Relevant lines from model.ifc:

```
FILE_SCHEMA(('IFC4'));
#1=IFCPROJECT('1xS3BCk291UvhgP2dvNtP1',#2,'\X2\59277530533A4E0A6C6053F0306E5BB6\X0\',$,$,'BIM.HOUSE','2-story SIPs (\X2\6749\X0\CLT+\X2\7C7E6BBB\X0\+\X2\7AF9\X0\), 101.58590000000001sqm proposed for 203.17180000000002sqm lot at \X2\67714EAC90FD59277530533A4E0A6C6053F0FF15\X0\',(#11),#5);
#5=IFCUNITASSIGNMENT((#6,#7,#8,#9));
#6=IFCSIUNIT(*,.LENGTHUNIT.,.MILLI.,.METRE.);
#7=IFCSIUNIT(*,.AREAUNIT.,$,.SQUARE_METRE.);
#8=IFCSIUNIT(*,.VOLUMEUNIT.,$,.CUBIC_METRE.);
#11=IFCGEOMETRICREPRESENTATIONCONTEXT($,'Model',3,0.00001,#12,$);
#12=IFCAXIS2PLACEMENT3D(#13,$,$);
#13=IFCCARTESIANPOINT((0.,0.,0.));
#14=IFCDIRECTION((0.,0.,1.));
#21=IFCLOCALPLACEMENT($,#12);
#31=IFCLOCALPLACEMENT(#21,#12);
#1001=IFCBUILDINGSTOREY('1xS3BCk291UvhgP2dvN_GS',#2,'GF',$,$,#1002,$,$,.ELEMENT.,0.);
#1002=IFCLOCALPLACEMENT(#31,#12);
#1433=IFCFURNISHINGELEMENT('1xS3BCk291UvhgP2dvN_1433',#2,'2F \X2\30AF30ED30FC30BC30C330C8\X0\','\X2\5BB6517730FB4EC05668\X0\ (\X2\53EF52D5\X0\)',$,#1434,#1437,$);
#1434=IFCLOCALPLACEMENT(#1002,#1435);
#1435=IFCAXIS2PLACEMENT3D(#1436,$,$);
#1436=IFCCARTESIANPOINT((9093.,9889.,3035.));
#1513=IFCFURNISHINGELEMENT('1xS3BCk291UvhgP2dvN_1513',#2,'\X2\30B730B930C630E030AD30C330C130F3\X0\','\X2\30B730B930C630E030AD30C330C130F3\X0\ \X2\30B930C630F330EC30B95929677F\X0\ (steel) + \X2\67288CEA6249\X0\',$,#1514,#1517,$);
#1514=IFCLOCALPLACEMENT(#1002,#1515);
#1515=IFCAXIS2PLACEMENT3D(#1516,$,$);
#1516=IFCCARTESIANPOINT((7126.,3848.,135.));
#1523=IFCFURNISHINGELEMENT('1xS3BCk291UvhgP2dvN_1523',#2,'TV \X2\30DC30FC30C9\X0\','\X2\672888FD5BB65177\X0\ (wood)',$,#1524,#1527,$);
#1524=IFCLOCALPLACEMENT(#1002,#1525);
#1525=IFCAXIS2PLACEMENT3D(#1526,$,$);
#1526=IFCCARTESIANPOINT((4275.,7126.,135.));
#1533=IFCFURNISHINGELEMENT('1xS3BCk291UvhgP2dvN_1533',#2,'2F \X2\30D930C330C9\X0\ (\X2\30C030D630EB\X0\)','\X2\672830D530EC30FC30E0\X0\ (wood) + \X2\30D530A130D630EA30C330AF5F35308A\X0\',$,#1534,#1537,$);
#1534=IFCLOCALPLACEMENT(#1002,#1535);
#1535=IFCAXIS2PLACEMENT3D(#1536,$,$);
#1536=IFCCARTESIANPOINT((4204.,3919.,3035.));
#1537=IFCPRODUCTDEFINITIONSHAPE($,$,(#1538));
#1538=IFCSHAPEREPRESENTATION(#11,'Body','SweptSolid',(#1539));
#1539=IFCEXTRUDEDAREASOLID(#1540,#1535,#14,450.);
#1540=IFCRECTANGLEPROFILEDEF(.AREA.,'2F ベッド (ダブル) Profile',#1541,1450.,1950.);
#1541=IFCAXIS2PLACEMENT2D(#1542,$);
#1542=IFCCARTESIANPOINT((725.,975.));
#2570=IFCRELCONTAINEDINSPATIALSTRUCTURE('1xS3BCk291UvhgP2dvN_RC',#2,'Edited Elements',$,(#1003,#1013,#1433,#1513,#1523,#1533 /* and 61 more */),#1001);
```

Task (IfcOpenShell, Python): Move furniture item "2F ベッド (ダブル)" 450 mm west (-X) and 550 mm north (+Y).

```python
import ifcopenshell
import ifcopenshell.api.geometry
import ifcopenshell.util.placement

model = ifcopenshell.open("model.ifc")

item = model.by_guid("1xS3BCk291UvhgP2dvN_1533")
matrix = ifcopenshell.util.placement.get_local_placement(item.ObjectPlacement)
matrix[0, 3] -= 450.0
matrix[1, 3] += 550.0
ifcopenshell.api.geometry.edit_object_placement(model, product=item, matrix=matrix, is_si=False)

print(ifcopenshell.util.placement.get_local_placement(item.ObjectPlacement).round(3) + 0.0)

model.write("model_rev.ifc")
```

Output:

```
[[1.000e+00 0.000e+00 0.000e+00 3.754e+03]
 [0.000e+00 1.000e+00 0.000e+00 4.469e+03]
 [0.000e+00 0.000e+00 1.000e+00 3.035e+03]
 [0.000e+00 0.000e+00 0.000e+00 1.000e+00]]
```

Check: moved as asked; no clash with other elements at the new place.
